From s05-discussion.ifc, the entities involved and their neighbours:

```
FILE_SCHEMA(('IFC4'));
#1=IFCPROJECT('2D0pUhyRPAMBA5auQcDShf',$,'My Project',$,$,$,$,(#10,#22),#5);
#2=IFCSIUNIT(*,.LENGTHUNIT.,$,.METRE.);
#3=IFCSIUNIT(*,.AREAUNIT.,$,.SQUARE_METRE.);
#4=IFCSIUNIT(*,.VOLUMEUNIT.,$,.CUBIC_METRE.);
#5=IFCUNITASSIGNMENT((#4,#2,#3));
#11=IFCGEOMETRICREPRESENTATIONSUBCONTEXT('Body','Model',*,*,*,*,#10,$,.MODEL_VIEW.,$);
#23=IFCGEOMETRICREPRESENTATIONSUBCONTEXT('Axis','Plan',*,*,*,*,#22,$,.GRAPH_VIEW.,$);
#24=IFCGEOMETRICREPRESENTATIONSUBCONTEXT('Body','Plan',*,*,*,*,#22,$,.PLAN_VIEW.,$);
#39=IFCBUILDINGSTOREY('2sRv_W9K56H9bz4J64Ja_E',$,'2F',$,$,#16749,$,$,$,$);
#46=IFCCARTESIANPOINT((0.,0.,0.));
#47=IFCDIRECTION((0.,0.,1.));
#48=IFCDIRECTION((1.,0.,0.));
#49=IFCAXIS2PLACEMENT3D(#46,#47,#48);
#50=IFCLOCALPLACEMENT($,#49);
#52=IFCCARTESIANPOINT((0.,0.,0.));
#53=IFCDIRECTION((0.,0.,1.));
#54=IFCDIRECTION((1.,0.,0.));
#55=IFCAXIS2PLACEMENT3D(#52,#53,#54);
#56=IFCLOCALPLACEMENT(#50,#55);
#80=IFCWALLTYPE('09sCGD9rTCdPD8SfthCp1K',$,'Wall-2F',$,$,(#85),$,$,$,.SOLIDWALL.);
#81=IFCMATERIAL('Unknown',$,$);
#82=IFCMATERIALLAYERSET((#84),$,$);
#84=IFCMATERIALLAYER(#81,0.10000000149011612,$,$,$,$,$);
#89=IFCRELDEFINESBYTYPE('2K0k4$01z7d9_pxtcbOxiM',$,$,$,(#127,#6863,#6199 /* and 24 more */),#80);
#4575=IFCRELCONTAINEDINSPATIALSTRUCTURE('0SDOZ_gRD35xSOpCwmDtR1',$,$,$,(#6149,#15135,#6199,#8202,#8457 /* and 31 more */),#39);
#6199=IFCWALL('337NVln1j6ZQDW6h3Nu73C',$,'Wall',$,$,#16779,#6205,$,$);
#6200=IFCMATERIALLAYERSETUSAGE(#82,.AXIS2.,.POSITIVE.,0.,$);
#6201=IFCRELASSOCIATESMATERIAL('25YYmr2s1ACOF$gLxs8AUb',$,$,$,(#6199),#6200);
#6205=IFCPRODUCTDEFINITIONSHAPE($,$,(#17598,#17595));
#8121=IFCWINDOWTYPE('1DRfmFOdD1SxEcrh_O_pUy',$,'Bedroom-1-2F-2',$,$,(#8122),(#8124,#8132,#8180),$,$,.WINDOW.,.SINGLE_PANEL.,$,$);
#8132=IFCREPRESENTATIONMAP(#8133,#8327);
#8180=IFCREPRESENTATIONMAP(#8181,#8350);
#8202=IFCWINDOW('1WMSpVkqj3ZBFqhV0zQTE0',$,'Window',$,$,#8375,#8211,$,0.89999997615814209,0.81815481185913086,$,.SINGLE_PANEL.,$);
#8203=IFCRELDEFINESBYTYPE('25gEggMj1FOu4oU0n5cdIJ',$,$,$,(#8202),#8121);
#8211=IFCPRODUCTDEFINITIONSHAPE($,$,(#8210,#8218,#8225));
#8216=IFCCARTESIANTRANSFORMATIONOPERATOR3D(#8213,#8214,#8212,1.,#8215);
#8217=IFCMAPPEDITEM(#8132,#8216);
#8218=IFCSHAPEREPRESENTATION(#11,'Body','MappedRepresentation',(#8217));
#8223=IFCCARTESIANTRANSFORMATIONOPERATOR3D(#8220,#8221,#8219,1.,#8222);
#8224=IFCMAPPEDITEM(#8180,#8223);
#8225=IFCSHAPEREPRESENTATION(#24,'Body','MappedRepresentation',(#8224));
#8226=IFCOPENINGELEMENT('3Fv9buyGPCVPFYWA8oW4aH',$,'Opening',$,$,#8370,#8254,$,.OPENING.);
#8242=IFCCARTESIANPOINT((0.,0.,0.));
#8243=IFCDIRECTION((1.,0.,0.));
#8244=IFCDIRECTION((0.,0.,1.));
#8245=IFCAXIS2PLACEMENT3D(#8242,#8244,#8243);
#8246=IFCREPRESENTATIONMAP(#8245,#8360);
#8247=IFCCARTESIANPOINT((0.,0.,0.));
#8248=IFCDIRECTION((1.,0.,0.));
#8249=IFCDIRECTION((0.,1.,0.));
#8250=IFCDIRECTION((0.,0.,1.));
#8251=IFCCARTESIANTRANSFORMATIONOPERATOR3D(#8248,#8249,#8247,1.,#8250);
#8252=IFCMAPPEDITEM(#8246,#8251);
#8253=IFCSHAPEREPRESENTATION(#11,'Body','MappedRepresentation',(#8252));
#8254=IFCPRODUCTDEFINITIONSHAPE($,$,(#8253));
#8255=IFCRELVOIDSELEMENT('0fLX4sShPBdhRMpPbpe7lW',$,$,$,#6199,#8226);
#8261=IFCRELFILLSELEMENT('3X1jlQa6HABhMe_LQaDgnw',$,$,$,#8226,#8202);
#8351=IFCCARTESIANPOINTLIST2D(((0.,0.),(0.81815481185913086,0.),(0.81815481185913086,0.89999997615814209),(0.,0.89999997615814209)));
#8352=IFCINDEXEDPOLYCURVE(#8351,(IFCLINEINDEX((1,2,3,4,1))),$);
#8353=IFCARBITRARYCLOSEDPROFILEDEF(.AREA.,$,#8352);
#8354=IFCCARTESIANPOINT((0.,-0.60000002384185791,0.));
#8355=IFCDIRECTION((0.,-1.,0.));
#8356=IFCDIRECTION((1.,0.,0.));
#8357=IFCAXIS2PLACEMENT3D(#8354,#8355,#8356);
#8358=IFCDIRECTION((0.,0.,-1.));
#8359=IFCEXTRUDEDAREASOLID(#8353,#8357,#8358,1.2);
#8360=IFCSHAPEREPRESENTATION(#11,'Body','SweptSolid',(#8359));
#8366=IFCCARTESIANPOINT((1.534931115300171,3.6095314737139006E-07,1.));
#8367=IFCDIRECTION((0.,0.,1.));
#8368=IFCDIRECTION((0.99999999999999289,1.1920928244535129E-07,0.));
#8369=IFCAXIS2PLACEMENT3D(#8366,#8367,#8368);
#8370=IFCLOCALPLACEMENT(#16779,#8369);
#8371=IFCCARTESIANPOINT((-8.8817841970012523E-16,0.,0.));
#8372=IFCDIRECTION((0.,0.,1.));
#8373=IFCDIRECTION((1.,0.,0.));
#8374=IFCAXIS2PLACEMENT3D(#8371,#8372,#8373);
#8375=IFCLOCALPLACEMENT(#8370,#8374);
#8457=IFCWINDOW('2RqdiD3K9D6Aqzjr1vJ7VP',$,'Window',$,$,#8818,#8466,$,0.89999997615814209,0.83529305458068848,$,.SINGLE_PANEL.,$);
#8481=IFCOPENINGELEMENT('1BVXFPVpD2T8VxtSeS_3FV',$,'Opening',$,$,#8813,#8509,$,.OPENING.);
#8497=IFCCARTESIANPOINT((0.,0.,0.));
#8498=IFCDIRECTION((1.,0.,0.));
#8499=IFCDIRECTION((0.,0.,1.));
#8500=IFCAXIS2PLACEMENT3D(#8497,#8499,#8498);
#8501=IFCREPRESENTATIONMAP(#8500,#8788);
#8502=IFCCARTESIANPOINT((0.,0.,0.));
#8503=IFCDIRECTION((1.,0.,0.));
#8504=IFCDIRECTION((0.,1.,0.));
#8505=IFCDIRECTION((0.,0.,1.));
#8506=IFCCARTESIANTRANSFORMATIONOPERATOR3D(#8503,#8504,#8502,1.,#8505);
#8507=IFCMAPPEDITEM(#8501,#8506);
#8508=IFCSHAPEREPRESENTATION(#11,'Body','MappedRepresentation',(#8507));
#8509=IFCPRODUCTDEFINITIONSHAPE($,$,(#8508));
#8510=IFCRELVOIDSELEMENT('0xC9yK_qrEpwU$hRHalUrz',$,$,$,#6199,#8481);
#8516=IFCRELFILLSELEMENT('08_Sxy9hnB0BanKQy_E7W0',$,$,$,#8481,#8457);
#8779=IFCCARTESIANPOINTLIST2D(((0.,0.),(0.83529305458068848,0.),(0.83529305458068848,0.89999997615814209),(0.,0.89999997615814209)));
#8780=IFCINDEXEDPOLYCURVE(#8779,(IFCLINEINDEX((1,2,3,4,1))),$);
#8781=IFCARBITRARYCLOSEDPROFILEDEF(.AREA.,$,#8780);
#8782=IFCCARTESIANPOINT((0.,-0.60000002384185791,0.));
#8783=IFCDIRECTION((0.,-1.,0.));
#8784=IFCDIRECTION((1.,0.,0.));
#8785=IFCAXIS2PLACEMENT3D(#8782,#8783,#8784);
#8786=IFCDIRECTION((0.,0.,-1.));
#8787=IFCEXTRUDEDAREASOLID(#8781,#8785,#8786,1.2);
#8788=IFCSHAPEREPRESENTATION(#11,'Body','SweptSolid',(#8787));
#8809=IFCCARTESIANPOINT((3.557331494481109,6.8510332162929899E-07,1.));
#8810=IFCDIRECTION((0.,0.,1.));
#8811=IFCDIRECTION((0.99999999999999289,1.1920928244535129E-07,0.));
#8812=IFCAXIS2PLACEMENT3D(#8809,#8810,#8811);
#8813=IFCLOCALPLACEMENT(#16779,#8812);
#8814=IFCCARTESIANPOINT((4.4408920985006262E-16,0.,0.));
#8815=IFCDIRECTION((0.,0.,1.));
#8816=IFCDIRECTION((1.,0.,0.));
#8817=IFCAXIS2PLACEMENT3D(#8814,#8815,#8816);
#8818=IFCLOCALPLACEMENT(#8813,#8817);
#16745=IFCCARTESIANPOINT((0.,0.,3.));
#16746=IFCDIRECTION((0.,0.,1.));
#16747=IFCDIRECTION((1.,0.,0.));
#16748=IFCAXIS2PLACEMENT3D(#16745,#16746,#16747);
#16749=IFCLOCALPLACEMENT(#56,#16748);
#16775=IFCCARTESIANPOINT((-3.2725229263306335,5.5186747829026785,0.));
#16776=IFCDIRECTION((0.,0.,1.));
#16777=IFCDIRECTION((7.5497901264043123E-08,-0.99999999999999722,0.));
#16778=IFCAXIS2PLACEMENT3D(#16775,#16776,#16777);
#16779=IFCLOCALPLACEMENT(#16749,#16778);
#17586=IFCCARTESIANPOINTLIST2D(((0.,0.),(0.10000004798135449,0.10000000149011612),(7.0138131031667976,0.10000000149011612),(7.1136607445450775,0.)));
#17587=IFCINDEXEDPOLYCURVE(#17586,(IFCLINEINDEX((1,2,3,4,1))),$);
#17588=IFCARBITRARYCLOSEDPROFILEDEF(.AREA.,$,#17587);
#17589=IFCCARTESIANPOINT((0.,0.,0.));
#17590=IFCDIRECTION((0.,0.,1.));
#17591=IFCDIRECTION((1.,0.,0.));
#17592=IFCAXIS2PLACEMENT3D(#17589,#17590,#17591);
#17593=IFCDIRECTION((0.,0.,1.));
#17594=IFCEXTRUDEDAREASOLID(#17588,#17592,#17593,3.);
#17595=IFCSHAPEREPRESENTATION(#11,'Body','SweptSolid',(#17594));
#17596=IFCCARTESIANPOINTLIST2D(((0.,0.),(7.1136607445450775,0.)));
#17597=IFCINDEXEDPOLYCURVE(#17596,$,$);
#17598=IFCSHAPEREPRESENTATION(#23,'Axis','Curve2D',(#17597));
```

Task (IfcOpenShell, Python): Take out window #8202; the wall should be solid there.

```python
import ifcopenshell
import ifcopenshell.api.feature
import ifcopenshell.api.root
import ifcopenshell.geom
import ifcopenshell.util.shape

model = ifcopenshell.open("s05-discussion.ifc")
settings = ifcopenshell.geom.settings()


def volume(element):
    """Net volume in cubic metres, openings subtracted."""
    shape = ifcopenshell.geom.create_shape(settings, element)
    return ifcopenshell.util.shape.get_volume(shape.geometry)


window = model.by_id(8202)
opening = window.FillsVoids[0].RelatingOpeningElement
wall = opening.VoidsElements[0].RelatingBuildingElement
before = volume(wall)

ifcopenshell.api.root.remove_product(model, product=window)
ifcopenshell.api.feature.remove_feature(model, feature=opening)

after = volume(wall)

print(f"wall volume {before:.3f} -> {after:.3f} m3")

model.write("s05-discussion_edited.ifc")
```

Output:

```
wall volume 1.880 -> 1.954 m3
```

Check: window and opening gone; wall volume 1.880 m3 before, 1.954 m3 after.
